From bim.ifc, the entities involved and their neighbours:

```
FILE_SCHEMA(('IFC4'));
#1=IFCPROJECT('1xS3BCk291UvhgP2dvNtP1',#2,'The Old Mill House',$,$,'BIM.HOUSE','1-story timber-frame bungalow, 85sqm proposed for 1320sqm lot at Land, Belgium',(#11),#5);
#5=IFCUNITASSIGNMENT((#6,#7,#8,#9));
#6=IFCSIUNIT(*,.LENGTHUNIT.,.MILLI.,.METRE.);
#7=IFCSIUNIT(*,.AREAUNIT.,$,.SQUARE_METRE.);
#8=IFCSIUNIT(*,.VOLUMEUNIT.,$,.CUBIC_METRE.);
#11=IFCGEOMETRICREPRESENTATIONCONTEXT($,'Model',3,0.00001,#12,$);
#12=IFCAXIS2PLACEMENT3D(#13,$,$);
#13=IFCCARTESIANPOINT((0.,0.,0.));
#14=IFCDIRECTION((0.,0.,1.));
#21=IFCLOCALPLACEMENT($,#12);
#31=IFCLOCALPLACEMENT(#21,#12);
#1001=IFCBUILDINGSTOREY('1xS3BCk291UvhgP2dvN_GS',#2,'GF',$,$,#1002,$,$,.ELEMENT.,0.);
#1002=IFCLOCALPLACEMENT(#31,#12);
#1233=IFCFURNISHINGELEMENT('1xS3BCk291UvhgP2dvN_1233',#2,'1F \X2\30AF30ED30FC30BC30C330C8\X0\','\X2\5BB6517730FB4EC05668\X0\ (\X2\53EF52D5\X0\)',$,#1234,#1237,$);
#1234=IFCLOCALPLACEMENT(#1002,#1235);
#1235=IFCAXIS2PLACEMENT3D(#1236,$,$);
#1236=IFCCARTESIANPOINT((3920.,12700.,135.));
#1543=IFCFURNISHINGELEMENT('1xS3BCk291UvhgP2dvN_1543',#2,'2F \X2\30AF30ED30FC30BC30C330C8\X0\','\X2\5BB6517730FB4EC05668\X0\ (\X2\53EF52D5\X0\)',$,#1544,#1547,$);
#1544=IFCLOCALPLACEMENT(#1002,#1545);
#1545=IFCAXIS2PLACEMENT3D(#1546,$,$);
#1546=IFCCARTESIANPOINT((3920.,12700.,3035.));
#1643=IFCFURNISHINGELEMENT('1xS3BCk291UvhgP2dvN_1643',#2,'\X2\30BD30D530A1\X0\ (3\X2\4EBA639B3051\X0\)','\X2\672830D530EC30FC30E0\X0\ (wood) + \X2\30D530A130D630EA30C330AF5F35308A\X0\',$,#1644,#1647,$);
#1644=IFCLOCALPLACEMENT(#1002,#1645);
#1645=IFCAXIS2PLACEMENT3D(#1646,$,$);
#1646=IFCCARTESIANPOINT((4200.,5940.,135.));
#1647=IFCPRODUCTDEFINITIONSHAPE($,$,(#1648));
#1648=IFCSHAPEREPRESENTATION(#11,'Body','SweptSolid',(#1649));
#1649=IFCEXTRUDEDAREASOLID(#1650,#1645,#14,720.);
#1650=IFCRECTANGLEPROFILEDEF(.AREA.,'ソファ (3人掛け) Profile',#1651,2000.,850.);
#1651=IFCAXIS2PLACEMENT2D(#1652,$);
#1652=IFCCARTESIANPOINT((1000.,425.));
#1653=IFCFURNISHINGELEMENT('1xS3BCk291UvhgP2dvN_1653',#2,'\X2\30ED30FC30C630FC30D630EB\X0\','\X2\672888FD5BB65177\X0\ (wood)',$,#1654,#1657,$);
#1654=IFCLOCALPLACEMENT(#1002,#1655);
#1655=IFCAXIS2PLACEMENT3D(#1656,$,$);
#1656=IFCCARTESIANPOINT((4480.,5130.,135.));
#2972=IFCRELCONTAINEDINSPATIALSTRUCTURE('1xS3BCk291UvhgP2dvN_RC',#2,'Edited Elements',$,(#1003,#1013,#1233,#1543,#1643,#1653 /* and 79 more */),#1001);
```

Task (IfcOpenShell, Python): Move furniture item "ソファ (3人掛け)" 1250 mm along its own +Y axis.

```python
import ifcopenshell
import ifcopenshell.api.geometry
import ifcopenshell.util.placement

model = ifcopenshell.open("bim.ifc")

item = model.by_guid("1xS3BCk291UvhgP2dvN_1643")
matrix = ifcopenshell.util.placement.get_local_placement(item.ObjectPlacement)
matrix[:3, 3] += matrix[:3, 1] * 1250.0
ifcopenshell.api.geometry.edit_object_placement(model, product=item, matrix=matrix, is_si=False)

print(ifcopenshell.util.placement.get_local_placement(item.ObjectPlacement).round(3) + 0.0)

model.write("bim_updated.ifc")
```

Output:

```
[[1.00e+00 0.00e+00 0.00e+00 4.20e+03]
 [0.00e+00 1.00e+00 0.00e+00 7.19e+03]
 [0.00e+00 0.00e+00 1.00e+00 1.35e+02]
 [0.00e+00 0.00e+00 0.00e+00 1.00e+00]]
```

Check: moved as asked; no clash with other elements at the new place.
